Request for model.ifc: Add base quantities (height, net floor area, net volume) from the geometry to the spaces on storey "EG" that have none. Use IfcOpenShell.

First a look at what the model holds.

```python
import ifcopenshell
import ifcopenshell.util.element
import ifcopenshell.util.unit

model = ifcopenshell.open("model.ifc")
print(model.schema)
for unit_type in ("LENGTHUNIT", "AREAUNIT", "VOLUMEUNIT"):
    print(unit_type, ifcopenshell.util.unit.calculate_unit_scale(model, unit_type))
storey = next(s for s in model.by_type("IfcBuildingStorey") if s.Name == "EG")
spaces = [e for e in ifcopenshell.util.element.get_decomposition(storey) if e.is_a("IfcSpace")]
for e in sorted(spaces, key=lambda e: e.id()):
    print(e.id(), e.is_a(), e.Name, list(ifcopenshell.util.element.get_psets(e, qtos_only=True)), sep=" | ")
```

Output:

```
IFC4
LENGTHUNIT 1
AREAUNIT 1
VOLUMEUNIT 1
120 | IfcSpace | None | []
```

```python
import ifcopenshell
import ifcopenshell.api.pset
import ifcopenshell.geom
import ifcopenshell.util.element
import ifcopenshell.util.shape
import ifcopenshell.util.unit

model = ifcopenshell.open("model.ifc")
unit_scale = ifcopenshell.util.unit.calculate_unit_scale(model)
area_scale = ifcopenshell.util.unit.calculate_unit_scale(model, "AREAUNIT")
volume_scale = ifcopenshell.util.unit.calculate_unit_scale(model, "VOLUMEUNIT")
settings = ifcopenshell.geom.settings()

storey = next(s for s in model.by_type("IfcBuildingStorey") if s.Name == "EG")
spaces = [e for e in ifcopenshell.util.element.get_decomposition(storey) if e.is_a("IfcSpace")]

for e in sorted(spaces, key=lambda e: e.id()):
    if ifcopenshell.util.element.get_psets(e, qtos_only=True, should_inherit=False):
        continue
    # Geometry comes back in metres, in the element's own axes.
    shape = ifcopenshell.geom.create_shape(settings, e)
    values = {
        "Height": ifcopenshell.util.shape.get_z(shape.geometry) / unit_scale,
        "NetFloorArea": ifcopenshell.util.shape.get_footprint_area(shape.geometry) / area_scale,
        "NetVolume": ifcopenshell.util.shape.get_volume(shape.geometry) / volume_scale,
    }
    qto = ifcopenshell.api.pset.add_qto(model, product=e, name="Qto_SpaceBaseQuantities")
    ifcopenshell.api.pset.edit_qto(model, qto=qto, properties=values)
    print(e.id(), {k: round(v, 3) for k, v in values.items()})

model.write("model_edited.ifc")
```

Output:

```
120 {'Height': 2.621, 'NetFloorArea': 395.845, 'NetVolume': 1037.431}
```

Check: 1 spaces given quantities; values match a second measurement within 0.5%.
